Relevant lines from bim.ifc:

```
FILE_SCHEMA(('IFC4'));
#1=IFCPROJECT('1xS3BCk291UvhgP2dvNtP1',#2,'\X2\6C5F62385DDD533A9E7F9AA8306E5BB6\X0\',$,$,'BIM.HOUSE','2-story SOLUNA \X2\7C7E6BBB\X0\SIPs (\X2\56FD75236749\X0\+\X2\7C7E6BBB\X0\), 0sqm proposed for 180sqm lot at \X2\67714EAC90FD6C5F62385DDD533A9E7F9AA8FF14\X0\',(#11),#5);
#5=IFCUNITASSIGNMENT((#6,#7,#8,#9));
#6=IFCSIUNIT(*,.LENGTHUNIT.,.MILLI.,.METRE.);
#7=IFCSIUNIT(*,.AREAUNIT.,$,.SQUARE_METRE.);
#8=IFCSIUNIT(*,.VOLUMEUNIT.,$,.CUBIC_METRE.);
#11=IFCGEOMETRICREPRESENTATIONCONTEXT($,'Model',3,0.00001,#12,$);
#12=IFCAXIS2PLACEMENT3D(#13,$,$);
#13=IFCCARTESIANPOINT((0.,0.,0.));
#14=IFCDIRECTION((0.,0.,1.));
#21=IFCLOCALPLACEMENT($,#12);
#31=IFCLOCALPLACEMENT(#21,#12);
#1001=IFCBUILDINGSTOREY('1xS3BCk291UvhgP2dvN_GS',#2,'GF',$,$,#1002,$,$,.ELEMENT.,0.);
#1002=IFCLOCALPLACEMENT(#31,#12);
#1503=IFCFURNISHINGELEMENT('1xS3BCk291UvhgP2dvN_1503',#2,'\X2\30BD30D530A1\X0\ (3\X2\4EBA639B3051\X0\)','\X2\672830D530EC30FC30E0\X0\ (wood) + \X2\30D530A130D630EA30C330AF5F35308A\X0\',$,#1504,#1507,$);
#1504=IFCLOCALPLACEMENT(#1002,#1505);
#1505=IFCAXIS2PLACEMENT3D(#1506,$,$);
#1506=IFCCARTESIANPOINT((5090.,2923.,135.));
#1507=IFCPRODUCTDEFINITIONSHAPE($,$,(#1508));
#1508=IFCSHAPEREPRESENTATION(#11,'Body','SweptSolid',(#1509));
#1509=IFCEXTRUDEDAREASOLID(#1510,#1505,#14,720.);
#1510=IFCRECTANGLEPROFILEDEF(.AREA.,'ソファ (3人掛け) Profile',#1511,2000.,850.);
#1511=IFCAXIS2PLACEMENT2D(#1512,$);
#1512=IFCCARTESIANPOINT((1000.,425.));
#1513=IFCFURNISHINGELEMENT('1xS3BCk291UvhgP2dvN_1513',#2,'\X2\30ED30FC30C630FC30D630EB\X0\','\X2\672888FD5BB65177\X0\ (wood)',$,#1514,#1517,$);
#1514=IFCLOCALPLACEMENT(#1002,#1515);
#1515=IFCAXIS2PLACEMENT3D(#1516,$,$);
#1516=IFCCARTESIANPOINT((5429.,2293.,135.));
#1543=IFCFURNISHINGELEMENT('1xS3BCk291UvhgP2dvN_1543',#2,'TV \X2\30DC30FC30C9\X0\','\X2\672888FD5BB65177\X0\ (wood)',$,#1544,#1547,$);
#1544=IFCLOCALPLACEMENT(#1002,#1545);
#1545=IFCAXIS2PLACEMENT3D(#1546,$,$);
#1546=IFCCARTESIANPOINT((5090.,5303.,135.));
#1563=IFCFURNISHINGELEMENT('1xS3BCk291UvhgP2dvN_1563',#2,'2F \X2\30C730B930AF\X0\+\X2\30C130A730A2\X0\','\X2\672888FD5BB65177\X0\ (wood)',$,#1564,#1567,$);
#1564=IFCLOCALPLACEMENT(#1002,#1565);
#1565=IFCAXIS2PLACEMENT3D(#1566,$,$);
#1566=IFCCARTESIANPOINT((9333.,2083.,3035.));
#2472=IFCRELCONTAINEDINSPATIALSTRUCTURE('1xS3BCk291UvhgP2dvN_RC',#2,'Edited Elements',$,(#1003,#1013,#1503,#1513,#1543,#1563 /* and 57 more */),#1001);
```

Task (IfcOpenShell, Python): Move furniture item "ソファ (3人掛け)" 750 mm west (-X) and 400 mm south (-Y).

```python
import ifcopenshell
import ifcopenshell.api.geometry
import ifcopenshell.util.placement
import ifcopenshell.util.unit

model = ifcopenshell.open("bim.ifc")
unit_scale = ifcopenshell.util.unit.calculate_unit_scale(model)

item = model.by_guid("1xS3BCk291UvhgP2dvN_1503")
matrix = ifcopenshell.util.placement.get_local_placement(item.ObjectPlacement)
matrix[0, 3] -= 0.75 / unit_scale
matrix[1, 3] -= 0.4 / unit_scale
ifcopenshell.api.geometry.edit_object_placement(model, product=item, matrix=matrix, is_si=False)

print(ifcopenshell.util.placement.get_local_placement(item.ObjectPlacement).round(3) + 0.0)

model.write("bim_v2.ifc")
```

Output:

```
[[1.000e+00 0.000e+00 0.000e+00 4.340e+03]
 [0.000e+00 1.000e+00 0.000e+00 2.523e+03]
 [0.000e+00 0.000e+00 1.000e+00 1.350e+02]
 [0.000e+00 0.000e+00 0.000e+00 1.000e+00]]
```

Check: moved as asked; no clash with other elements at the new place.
